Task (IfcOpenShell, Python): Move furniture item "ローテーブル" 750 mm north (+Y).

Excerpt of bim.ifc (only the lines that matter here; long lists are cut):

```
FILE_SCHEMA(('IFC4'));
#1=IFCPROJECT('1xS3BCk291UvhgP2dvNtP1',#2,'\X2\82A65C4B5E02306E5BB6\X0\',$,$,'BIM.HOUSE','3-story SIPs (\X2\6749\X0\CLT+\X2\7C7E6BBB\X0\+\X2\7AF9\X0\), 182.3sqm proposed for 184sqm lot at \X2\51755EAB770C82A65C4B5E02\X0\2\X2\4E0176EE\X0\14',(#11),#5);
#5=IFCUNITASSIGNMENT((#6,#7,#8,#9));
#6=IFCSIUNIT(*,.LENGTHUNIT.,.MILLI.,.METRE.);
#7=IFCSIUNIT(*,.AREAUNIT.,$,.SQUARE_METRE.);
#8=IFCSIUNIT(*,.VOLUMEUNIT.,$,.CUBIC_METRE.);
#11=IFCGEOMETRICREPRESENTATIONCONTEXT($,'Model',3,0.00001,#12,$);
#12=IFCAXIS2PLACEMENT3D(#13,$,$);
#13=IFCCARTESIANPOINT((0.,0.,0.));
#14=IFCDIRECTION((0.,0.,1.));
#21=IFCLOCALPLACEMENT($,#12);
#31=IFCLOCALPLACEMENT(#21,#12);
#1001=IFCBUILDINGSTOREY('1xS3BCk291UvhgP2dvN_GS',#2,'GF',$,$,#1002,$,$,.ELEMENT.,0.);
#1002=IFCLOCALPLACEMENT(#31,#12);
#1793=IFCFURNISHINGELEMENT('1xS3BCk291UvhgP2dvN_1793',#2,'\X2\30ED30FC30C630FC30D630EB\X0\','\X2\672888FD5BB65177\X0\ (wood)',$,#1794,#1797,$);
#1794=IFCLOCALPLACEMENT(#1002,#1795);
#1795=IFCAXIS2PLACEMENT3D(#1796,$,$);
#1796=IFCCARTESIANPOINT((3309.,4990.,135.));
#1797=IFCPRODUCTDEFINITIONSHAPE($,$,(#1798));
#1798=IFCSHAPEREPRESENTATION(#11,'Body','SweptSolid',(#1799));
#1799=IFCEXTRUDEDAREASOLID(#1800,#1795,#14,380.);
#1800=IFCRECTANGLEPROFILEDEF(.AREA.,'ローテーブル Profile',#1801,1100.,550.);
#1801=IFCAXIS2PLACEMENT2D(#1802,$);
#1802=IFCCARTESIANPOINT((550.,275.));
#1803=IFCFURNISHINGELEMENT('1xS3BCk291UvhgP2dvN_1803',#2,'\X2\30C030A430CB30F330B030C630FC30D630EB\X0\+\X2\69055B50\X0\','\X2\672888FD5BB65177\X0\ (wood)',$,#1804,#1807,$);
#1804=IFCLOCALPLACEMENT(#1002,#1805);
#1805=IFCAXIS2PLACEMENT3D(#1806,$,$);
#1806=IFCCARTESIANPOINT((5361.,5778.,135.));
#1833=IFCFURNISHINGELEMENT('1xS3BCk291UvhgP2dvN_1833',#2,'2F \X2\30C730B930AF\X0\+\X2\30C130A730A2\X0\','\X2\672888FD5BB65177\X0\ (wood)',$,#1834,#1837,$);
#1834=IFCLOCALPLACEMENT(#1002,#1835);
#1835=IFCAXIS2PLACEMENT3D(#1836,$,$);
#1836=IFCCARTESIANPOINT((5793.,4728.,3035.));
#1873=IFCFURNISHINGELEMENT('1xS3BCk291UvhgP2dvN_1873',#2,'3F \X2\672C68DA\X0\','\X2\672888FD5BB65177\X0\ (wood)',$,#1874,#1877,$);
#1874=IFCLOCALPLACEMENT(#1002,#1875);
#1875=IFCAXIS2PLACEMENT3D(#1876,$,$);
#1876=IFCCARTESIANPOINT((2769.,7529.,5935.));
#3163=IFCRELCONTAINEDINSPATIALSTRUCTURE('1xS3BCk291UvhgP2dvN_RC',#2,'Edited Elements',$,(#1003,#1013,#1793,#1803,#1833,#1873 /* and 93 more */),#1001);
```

```python
import ifcopenshell
import ifcopenshell.api.geometry
import ifcopenshell.util.placement
import ifcopenshell.util.unit

model = ifcopenshell.open("bim.ifc")
unit_scale = ifcopenshell.util.unit.calculate_unit_scale(model)

item = model.by_id(1793)
matrix = ifcopenshell.util.placement.get_local_placement(item.ObjectPlacement)
matrix[1, 3] += 0.75 / unit_scale
ifcopenshell.api.geometry.edit_object_placement(model, product=item, matrix=matrix, is_si=False)

print(ifcopenshell.util.placement.get_local_placement(item.ObjectPlacement).round(3) + 0.0)

model.write("bim_v2.ifc")
```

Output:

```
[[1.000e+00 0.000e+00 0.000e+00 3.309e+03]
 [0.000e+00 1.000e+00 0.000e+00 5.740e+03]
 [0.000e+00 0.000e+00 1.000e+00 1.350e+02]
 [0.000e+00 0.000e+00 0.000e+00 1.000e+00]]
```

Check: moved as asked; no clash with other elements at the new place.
